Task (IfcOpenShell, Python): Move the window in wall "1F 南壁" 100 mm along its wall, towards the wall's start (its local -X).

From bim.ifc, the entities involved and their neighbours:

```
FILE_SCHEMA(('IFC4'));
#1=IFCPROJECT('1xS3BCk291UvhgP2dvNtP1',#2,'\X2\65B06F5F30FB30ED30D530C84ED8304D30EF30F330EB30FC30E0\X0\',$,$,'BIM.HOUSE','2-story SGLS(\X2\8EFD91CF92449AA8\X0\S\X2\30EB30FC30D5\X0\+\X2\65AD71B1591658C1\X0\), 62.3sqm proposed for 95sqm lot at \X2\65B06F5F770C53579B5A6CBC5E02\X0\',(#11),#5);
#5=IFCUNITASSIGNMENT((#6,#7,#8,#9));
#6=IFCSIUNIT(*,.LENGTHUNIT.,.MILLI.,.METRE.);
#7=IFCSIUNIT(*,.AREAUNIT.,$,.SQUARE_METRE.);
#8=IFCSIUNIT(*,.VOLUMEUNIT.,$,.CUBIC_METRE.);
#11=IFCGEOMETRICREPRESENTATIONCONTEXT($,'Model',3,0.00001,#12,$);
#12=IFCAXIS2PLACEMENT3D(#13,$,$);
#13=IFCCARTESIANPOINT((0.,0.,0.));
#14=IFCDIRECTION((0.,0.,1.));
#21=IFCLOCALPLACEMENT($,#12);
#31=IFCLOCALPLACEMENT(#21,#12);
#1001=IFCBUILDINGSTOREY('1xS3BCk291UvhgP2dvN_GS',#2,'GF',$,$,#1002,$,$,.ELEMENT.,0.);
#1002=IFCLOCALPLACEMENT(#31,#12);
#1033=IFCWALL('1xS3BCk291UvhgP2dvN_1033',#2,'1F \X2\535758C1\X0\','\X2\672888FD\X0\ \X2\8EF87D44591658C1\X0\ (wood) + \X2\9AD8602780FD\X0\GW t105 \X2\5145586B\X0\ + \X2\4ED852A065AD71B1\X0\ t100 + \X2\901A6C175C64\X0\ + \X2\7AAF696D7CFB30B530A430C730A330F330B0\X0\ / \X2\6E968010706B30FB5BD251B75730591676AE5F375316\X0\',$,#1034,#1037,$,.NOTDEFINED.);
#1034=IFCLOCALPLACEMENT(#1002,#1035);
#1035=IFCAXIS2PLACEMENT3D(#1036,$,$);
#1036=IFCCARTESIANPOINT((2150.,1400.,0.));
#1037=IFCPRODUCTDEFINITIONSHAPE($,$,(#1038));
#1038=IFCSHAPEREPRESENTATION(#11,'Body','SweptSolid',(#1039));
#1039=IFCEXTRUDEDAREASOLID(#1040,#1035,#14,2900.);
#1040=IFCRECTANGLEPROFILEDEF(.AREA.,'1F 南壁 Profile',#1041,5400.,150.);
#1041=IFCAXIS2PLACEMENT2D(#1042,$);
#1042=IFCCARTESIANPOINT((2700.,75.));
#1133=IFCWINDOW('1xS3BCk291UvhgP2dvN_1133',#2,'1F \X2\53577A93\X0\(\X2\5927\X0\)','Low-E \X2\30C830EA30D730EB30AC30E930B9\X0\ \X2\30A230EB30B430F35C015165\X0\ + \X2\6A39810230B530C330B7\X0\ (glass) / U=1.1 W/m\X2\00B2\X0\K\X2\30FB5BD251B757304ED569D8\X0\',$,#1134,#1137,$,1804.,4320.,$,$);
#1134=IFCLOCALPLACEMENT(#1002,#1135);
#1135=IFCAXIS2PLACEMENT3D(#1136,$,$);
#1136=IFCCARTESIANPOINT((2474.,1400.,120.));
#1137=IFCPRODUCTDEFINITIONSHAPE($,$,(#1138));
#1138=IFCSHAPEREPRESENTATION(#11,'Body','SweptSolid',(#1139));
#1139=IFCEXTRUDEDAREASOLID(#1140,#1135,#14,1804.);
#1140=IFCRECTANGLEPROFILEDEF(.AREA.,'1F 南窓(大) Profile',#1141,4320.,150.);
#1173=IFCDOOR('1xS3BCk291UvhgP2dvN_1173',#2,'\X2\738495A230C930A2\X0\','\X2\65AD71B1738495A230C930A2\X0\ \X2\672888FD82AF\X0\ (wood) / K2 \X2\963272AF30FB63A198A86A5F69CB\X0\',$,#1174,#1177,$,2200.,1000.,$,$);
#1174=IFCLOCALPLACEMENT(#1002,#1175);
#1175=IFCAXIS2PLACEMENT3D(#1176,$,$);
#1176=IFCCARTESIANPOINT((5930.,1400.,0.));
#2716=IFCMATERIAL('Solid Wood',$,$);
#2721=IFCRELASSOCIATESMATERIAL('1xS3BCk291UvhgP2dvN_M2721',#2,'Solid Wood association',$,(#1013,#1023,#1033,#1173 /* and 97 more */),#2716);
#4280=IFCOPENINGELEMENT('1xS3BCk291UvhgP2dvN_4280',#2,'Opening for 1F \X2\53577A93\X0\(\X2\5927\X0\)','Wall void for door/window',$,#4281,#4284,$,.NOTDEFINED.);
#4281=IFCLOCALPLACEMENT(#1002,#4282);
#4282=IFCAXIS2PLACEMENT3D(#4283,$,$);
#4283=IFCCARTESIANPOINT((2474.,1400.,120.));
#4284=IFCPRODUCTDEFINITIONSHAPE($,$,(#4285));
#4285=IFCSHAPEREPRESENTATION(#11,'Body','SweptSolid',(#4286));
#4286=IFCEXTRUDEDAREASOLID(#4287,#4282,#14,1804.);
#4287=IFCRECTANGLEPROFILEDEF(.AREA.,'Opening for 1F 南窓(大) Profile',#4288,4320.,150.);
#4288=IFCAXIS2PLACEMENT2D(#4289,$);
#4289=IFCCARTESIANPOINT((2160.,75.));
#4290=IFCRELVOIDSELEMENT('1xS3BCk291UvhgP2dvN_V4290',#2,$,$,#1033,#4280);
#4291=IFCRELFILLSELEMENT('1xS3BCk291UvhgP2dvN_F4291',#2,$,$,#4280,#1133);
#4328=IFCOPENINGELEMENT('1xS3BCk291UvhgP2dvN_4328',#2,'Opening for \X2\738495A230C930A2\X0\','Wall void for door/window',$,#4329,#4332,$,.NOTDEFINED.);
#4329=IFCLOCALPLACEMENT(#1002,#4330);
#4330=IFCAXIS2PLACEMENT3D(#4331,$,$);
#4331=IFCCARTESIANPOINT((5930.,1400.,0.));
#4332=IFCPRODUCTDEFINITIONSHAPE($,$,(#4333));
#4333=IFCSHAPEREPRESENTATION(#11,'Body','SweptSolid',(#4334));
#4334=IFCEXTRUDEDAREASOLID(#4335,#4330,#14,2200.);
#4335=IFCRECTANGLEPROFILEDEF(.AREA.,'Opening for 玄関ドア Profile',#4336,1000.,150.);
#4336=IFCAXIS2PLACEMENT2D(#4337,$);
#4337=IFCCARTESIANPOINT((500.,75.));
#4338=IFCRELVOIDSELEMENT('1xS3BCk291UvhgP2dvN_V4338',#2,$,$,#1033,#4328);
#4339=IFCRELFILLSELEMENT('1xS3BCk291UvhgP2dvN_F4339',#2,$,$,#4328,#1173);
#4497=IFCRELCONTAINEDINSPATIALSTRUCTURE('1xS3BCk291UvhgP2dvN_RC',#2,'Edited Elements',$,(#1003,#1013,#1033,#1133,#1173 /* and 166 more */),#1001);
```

```python
import ifcopenshell
import ifcopenshell.api.geometry
import ifcopenshell.util.placement
import ifcopenshell.util.unit

model = ifcopenshell.open("bim.ifc")
unit_scale = ifcopenshell.util.unit.calculate_unit_scale(model)

window = model.by_guid("1xS3BCk291UvhgP2dvN_1133")
opening = window.FillsVoids[0].RelatingOpeningElement
wall = opening.VoidsElements[0].RelatingBuildingElement

wall_matrix = ifcopenshell.util.placement.get_local_placement(wall.ObjectPlacement)
shift = wall_matrix[:3, 0] * -0.1 / unit_scale
before = ifcopenshell.util.placement.get_local_placement(window.ObjectPlacement)[:3, 3].copy()

# The window is not placed relative to its opening, so move both.
for product in (opening, window):
    matrix = ifcopenshell.util.placement.get_local_placement(product.ObjectPlacement)
    matrix[:3, 3] += shift
    ifcopenshell.api.geometry.edit_object_placement(model, product=product, matrix=matrix, is_si=False)

after = ifcopenshell.util.placement.get_local_placement(window.ObjectPlacement)[:3, 3]
print("window moved by", (after - before).round(3) + 0.0)

model.write("bim-out.ifc")
```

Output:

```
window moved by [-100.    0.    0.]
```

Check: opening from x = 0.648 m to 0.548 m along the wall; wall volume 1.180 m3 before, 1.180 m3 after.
